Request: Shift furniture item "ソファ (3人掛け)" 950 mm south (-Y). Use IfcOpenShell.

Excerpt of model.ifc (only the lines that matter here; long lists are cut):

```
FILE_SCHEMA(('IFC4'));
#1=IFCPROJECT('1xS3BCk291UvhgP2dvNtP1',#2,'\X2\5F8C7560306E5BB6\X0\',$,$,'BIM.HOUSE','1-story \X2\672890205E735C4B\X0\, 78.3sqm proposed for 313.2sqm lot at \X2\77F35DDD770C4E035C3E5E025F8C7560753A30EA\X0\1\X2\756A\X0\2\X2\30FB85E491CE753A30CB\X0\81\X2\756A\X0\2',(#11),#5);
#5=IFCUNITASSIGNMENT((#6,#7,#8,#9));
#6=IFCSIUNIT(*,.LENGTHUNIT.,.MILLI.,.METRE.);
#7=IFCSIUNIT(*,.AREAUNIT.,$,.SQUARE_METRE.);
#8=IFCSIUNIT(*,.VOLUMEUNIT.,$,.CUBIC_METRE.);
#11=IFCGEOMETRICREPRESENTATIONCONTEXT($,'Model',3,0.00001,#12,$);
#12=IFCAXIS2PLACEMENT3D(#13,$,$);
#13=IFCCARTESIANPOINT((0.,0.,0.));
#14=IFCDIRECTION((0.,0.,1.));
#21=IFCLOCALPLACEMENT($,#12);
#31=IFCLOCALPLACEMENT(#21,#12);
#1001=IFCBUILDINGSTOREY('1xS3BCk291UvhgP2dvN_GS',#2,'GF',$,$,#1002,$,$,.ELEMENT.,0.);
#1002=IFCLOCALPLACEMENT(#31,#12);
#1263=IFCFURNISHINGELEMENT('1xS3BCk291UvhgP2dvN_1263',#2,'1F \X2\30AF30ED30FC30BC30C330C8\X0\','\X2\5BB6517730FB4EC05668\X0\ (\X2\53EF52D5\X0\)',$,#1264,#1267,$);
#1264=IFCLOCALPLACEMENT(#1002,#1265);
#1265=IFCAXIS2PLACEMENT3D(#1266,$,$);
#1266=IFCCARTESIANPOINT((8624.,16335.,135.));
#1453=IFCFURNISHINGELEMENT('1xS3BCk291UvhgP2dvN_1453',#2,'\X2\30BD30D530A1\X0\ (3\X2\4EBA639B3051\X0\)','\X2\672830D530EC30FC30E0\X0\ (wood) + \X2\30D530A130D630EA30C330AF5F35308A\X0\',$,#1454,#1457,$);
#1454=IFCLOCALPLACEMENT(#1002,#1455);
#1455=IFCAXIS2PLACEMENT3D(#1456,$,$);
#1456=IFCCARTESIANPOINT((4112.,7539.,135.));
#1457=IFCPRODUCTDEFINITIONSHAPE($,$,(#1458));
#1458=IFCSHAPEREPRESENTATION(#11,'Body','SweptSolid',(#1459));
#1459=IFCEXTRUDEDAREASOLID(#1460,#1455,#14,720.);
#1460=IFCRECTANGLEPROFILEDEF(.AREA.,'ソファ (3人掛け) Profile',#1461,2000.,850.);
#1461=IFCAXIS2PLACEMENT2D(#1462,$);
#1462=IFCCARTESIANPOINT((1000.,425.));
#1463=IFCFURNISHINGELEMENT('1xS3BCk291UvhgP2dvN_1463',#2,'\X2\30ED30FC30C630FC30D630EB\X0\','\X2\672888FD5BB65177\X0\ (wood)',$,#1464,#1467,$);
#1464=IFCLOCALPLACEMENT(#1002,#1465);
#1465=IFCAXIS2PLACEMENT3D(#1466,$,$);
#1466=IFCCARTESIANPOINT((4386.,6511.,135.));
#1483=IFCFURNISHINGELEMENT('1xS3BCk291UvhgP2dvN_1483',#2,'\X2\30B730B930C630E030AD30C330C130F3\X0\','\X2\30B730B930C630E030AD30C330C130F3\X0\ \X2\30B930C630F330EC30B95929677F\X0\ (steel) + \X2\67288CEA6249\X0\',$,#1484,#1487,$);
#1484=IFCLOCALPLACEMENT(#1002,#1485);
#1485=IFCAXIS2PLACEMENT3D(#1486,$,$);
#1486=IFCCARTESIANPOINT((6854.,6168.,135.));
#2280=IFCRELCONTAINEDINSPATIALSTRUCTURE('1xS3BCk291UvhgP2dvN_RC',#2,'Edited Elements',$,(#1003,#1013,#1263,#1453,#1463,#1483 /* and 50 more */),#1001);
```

```python
import ifcopenshell
import ifcopenshell.api.geometry
import ifcopenshell.util.placement

model = ifcopenshell.open("model.ifc")

item = model.by_id(1453)
matrix = ifcopenshell.util.placement.get_local_placement(item.ObjectPlacement)
matrix[1, 3] -= 950.0
ifcopenshell.api.geometry.edit_object_placement(model, product=item, matrix=matrix, is_si=False)

print(ifcopenshell.util.placement.get_local_placement(item.ObjectPlacement).round(3) + 0.0)

model.write("model-out.ifc")
```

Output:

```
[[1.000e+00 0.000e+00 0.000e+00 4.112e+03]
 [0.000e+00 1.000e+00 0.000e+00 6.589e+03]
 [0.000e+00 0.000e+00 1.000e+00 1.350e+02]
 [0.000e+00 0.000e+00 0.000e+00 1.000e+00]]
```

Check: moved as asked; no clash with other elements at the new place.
